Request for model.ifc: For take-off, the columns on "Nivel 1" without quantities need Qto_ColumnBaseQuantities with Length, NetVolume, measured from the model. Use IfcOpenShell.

First a look at what the model holds.

```python
import ifcopenshell
import ifcopenshell.util.element
import ifcopenshell.util.unit

model = ifcopenshell.open("model.ifc")
print(model.schema)
for unit_type in ("LENGTHUNIT", "AREAUNIT", "VOLUMEUNIT"):
    print(unit_type, ifcopenshell.util.unit.calculate_unit_scale(model, unit_type))
storey = next(s for s in model.by_type("IfcBuildingStorey") if s.Name == "Nivel 1")
columns = [e for e in ifcopenshell.util.element.get_decomposition(storey) if e.is_a("IfcColumn")]
for e in sorted(columns, key=lambda e: e.id()):
    print(e.id(), e.is_a(), e.Name, list(ifcopenshell.util.element.get_psets(e, qtos_only=True)), sep=" | ")
```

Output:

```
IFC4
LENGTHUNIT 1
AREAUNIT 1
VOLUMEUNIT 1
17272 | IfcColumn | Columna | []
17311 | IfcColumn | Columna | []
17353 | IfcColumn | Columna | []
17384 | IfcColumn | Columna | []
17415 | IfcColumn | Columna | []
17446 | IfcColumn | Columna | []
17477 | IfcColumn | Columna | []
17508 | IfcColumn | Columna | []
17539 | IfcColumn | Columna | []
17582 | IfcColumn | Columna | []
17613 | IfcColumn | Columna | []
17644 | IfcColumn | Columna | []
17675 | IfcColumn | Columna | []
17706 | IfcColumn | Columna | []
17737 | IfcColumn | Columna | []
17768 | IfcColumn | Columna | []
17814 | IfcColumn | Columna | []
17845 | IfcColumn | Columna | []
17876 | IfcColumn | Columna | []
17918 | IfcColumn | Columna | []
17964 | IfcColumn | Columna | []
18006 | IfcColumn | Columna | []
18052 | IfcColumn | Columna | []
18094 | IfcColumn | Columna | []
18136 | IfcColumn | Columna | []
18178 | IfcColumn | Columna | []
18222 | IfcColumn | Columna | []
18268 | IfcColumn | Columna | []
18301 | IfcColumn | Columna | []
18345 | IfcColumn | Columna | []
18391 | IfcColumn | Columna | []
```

```python
import ifcopenshell
import ifcopenshell.api.pset
import ifcopenshell.geom
import ifcopenshell.util.element
import ifcopenshell.util.shape
import ifcopenshell.util.unit

model = ifcopenshell.open("model.ifc")
unit_scale = ifcopenshell.util.unit.calculate_unit_scale(model)
volume_scale = ifcopenshell.util.unit.calculate_unit_scale(model, "VOLUMEUNIT")
settings = ifcopenshell.geom.settings()

storey = next(s for s in model.by_type("IfcBuildingStorey") if s.Name == "Nivel 1")
columns = [e for e in ifcopenshell.util.element.get_decomposition(storey) if e.is_a("IfcColumn")]

for e in sorted(columns, key=lambda e: e.id()):
    if ifcopenshell.util.element.get_psets(e, qtos_only=True, should_inherit=False):
        continue
    # Geometry comes back in metres, in the element's own axes.
    shape = ifcopenshell.geom.create_shape(settings, e)
    values = {
        "Length": ifcopenshell.util.shape.get_z(shape.geometry) / unit_scale,
        "NetVolume": ifcopenshell.util.shape.get_volume(shape.geometry) / volume_scale,
    }
    qto = ifcopenshell.api.pset.add_qto(model, product=e, name="Qto_ColumnBaseQuantities")
    ifcopenshell.api.pset.edit_qto(model, qto=qto, properties=values)
    print(e.id(), {k: round(v, 3) for k, v in values.items()})

model.write("model_rev.ifc")
```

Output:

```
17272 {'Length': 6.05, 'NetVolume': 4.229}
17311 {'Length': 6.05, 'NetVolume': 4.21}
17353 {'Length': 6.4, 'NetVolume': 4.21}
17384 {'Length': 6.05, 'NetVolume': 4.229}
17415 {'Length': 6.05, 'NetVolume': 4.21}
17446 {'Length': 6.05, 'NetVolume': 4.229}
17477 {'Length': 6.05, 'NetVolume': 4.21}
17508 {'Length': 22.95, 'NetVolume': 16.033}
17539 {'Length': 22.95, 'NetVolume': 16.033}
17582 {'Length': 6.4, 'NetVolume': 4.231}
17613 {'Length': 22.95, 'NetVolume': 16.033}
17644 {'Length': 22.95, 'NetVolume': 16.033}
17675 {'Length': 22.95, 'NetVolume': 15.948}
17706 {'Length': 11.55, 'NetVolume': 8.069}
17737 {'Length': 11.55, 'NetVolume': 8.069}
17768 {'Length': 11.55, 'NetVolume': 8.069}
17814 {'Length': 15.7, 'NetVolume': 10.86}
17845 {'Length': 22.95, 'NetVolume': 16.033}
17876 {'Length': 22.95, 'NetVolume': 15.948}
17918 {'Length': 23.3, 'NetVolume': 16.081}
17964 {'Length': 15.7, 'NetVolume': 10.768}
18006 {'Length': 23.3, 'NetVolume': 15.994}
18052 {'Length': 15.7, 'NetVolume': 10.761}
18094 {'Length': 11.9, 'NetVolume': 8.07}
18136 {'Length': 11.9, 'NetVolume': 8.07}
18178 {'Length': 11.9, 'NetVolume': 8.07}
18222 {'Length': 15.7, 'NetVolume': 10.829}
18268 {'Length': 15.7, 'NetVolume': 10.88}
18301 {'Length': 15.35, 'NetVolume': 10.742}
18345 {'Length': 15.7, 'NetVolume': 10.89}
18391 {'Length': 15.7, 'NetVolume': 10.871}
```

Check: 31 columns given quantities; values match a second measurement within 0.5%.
